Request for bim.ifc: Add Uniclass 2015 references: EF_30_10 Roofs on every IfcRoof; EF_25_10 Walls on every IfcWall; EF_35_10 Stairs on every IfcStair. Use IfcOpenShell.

First a look at what the model holds.

```python
import ifcopenshell

model = ifcopenshell.open("bim.ifc")
print(model.schema)
print("classifications:", [c.Name for c in model.by_type("IfcClassification")])
for ifc_class in ("IfcDoor", "IfcRoof", "IfcStair", "IfcWall", "IfcWindow"):
    print(ifc_class, len(model.by_type(ifc_class)))
```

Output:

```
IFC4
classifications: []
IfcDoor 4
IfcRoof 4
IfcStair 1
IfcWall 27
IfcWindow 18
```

```python
import ifcopenshell
import ifcopenshell.api.classification

model = ifcopenshell.open("bim.ifc")

system = ifcopenshell.api.classification.add_classification(model, classification="Uniclass 2015")

codes = {
    "IfcRoof": ("EF_30_10", "Roofs"),
    "IfcWall": ("EF_25_10", "Walls"),
    "IfcStair": ("EF_35_10", "Stairs"),
}
for ifc_class, (code, name) in codes.items():
    products = model.by_type(ifc_class)
    ifcopenshell.api.classification.add_reference(
        model, products=products, classification=system, identification=code, name=name
    )
    print(code, len(products))

model.write("bim_updated.ifc")
```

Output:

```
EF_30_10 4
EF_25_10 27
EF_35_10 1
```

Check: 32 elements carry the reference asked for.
